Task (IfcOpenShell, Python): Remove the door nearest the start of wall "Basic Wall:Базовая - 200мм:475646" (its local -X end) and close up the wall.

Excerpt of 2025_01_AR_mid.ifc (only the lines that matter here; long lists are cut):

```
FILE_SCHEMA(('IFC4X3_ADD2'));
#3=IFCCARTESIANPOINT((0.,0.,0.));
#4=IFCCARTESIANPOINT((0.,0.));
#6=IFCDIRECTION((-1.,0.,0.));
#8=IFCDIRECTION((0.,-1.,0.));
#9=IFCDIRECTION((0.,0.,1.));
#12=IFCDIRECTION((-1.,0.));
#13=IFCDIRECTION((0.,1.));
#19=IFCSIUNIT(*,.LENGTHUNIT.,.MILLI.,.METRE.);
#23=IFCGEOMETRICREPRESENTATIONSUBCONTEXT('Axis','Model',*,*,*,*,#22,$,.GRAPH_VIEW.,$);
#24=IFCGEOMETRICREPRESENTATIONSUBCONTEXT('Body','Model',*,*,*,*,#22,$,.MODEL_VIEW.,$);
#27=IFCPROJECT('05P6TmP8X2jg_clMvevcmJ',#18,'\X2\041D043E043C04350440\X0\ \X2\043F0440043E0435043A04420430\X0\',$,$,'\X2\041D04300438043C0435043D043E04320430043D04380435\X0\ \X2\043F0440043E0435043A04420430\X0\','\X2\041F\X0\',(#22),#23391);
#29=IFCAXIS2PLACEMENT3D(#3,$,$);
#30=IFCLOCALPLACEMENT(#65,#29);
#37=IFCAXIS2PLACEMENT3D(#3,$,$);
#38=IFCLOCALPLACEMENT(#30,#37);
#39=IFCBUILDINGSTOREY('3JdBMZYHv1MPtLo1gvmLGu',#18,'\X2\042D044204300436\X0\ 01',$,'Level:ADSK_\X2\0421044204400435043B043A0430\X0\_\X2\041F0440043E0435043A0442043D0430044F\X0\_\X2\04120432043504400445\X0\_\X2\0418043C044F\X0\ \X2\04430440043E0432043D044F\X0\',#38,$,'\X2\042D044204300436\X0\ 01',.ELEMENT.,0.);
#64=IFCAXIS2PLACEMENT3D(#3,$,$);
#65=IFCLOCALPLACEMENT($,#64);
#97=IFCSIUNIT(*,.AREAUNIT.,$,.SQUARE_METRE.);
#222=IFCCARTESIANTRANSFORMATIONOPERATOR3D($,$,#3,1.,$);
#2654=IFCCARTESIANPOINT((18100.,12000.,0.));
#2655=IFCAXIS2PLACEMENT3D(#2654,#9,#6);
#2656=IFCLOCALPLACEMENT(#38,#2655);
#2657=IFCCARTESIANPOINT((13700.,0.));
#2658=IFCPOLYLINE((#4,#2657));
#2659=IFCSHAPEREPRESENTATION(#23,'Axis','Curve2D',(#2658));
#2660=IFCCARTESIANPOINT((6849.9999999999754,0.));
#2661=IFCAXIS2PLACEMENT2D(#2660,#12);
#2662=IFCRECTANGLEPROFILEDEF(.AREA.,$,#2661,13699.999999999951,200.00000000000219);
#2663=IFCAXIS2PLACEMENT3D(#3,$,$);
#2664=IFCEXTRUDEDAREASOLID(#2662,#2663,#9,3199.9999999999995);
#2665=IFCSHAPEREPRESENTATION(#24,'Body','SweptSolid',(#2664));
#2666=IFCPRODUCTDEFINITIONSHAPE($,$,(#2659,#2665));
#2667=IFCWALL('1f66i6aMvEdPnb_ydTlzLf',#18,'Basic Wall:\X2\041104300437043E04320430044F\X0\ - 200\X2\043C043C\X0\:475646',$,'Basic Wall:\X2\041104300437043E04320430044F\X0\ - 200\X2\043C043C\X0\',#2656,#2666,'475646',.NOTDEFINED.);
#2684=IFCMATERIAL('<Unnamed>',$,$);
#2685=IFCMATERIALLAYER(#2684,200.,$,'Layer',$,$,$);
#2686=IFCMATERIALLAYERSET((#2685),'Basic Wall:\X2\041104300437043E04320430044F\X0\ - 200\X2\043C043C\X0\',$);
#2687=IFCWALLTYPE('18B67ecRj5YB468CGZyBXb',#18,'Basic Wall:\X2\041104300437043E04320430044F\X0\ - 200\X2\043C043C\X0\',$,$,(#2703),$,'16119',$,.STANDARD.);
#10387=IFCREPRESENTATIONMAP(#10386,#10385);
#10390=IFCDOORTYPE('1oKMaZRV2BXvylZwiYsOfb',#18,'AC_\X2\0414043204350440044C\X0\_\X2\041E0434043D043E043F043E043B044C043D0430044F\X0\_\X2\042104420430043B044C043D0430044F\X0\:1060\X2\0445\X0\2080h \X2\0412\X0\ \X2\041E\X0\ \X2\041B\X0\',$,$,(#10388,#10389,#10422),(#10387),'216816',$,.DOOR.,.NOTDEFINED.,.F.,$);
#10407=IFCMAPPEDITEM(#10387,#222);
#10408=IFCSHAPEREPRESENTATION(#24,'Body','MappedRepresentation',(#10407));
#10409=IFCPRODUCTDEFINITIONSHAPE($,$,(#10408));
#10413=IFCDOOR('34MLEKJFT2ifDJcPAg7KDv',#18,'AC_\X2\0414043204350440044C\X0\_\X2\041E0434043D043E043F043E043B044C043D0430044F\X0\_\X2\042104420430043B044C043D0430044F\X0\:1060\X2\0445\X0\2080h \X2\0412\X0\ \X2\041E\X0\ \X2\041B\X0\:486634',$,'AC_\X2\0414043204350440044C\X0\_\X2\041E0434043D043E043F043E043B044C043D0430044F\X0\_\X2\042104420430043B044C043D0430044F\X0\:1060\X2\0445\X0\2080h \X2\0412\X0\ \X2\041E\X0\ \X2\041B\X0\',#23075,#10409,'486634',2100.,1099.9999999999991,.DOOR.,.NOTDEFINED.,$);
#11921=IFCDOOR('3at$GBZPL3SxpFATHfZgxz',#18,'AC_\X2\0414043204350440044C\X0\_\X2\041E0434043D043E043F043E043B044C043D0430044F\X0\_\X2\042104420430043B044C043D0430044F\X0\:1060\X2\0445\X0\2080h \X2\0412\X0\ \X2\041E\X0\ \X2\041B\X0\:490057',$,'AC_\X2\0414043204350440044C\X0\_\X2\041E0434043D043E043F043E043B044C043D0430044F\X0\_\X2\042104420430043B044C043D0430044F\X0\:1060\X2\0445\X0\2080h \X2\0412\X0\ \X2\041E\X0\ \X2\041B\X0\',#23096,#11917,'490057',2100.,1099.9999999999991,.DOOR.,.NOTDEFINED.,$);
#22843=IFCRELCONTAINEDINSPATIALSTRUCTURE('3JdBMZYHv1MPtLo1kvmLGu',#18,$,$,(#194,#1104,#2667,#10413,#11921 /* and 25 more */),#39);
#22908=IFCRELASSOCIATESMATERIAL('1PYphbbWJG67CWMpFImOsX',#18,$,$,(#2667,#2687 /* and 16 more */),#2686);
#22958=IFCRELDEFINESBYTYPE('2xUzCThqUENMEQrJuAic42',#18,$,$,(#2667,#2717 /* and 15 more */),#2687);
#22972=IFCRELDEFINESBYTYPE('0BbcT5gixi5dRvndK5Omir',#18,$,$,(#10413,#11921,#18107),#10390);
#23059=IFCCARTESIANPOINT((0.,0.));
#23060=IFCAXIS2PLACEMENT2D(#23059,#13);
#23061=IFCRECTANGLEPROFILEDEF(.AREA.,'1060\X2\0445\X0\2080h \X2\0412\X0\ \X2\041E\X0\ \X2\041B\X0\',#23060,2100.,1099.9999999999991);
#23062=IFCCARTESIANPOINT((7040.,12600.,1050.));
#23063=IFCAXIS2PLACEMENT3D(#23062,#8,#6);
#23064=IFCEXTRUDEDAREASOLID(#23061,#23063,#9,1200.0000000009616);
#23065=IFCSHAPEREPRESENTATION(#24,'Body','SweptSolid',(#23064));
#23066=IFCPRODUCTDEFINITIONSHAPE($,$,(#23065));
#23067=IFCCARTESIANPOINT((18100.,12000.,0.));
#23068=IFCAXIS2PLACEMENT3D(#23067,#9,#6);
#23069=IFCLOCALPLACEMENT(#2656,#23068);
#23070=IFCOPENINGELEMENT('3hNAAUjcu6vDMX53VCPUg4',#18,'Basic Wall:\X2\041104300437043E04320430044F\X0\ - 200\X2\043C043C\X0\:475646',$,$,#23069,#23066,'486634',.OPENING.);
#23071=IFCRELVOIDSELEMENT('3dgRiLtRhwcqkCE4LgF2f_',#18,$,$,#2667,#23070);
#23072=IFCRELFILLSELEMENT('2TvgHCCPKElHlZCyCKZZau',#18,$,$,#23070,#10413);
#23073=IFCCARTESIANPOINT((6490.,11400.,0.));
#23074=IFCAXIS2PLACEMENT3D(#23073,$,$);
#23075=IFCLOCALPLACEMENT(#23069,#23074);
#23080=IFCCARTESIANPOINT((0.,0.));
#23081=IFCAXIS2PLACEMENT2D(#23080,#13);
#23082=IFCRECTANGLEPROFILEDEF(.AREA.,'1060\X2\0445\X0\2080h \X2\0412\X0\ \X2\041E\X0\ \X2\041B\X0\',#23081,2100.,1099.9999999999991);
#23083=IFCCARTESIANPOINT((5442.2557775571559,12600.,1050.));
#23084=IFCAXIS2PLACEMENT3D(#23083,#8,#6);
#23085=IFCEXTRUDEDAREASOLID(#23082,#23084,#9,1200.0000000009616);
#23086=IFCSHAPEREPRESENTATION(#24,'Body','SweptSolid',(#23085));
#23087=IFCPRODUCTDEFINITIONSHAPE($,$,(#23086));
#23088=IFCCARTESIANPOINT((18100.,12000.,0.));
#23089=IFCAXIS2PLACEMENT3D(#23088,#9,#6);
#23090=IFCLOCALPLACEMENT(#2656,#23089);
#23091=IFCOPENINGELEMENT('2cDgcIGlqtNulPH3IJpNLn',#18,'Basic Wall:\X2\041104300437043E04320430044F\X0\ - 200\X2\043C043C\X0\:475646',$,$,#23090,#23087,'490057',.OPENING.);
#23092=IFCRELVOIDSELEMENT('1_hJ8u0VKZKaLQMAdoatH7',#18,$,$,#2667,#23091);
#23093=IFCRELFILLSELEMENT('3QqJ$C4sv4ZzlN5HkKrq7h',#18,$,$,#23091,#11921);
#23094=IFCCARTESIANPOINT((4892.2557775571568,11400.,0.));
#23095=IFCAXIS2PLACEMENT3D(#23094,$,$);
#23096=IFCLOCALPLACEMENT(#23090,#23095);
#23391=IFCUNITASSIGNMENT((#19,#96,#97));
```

```python
import ifcopenshell
import ifcopenshell.api.feature
import ifcopenshell.api.root
import ifcopenshell.geom
import ifcopenshell.util.shape

model = ifcopenshell.open("2025_01_AR_mid.ifc")
settings = ifcopenshell.geom.settings()


def volume(element):
    """Net volume in cubic metres, openings subtracted."""
    shape = ifcopenshell.geom.create_shape(settings, element)
    return ifcopenshell.util.shape.get_volume(shape.geometry)


door = model.by_guid("34MLEKJFT2ifDJcPAg7KDv")
opening = door.FillsVoids[0].RelatingOpeningElement
wall = opening.VoidsElements[0].RelatingBuildingElement
before = volume(wall)

ifcopenshell.api.root.remove_product(model, product=door)
ifcopenshell.api.feature.remove_feature(model, feature=opening)

after = volume(wall)

print(f"wall volume {before:.3f} -> {after:.3f} m3")

model.write("2025_01_AR_mid_rev.ifc")
```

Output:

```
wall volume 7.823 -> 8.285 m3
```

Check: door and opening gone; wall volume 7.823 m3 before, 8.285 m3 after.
